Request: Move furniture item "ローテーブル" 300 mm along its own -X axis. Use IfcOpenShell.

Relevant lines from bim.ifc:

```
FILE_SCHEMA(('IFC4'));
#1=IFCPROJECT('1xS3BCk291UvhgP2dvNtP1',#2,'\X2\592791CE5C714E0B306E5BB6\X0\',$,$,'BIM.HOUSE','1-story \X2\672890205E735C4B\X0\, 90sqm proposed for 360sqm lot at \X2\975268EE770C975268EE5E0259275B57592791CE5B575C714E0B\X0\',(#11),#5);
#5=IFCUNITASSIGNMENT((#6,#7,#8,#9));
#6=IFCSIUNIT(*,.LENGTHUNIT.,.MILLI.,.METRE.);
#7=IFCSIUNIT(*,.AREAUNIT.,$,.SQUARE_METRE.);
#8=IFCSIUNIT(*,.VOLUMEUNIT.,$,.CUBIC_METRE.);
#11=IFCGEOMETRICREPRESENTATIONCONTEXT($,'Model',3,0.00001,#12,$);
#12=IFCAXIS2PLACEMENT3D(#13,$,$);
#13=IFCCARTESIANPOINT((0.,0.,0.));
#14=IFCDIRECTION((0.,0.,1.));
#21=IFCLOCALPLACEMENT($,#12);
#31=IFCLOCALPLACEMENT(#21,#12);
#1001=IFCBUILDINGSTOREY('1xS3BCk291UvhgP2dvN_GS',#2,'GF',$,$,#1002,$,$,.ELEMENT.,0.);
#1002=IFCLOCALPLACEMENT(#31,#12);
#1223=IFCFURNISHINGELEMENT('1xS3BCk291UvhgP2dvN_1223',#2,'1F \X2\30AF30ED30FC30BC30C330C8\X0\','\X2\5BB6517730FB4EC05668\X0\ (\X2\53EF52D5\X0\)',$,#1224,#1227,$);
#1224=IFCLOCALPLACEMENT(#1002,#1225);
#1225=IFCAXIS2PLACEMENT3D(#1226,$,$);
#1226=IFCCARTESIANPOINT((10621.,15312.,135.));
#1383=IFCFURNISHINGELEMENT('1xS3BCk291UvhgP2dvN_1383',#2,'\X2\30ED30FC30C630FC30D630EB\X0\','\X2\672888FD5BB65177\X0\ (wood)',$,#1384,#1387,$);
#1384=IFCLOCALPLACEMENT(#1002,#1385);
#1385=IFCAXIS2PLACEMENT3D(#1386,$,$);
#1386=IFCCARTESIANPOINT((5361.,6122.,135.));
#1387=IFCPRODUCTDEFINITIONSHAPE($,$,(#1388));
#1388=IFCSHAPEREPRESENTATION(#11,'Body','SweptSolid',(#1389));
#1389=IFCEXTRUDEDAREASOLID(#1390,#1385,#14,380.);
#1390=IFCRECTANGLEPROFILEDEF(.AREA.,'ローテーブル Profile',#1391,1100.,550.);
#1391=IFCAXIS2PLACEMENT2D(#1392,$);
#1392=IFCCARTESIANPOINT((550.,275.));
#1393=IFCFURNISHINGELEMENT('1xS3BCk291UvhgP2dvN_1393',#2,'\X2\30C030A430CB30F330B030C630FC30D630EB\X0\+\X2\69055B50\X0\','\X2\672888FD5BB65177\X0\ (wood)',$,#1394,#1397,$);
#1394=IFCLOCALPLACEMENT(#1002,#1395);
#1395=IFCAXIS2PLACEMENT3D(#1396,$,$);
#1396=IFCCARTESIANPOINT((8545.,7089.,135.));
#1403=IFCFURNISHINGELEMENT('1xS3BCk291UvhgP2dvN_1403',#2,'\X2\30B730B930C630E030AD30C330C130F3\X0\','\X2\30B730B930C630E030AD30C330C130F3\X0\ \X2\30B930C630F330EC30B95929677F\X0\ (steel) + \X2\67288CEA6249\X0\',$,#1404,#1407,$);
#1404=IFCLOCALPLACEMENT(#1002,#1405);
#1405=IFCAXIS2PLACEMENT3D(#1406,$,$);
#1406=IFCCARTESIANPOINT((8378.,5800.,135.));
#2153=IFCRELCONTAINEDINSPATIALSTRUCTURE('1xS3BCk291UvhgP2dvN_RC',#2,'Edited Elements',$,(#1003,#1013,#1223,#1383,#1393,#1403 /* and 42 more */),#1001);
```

```python
import ifcopenshell
import ifcopenshell.api.geometry
import ifcopenshell.util.placement

model = ifcopenshell.open("bim.ifc")

item = model.by_guid("1xS3BCk291UvhgP2dvN_1383")
matrix = ifcopenshell.util.placement.get_local_placement(item.ObjectPlacement)
matrix[:3, 3] -= matrix[:3, 0] * 300.0
ifcopenshell.api.geometry.edit_object_placement(model, product=item, matrix=matrix, is_si=False)

print(ifcopenshell.util.placement.get_local_placement(item.ObjectPlacement).round(3) + 0.0)

model.write("bim_edited.ifc")
```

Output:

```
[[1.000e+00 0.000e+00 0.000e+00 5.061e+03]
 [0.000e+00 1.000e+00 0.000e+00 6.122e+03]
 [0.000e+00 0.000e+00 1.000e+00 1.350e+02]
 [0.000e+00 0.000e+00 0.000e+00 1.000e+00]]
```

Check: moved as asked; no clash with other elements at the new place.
